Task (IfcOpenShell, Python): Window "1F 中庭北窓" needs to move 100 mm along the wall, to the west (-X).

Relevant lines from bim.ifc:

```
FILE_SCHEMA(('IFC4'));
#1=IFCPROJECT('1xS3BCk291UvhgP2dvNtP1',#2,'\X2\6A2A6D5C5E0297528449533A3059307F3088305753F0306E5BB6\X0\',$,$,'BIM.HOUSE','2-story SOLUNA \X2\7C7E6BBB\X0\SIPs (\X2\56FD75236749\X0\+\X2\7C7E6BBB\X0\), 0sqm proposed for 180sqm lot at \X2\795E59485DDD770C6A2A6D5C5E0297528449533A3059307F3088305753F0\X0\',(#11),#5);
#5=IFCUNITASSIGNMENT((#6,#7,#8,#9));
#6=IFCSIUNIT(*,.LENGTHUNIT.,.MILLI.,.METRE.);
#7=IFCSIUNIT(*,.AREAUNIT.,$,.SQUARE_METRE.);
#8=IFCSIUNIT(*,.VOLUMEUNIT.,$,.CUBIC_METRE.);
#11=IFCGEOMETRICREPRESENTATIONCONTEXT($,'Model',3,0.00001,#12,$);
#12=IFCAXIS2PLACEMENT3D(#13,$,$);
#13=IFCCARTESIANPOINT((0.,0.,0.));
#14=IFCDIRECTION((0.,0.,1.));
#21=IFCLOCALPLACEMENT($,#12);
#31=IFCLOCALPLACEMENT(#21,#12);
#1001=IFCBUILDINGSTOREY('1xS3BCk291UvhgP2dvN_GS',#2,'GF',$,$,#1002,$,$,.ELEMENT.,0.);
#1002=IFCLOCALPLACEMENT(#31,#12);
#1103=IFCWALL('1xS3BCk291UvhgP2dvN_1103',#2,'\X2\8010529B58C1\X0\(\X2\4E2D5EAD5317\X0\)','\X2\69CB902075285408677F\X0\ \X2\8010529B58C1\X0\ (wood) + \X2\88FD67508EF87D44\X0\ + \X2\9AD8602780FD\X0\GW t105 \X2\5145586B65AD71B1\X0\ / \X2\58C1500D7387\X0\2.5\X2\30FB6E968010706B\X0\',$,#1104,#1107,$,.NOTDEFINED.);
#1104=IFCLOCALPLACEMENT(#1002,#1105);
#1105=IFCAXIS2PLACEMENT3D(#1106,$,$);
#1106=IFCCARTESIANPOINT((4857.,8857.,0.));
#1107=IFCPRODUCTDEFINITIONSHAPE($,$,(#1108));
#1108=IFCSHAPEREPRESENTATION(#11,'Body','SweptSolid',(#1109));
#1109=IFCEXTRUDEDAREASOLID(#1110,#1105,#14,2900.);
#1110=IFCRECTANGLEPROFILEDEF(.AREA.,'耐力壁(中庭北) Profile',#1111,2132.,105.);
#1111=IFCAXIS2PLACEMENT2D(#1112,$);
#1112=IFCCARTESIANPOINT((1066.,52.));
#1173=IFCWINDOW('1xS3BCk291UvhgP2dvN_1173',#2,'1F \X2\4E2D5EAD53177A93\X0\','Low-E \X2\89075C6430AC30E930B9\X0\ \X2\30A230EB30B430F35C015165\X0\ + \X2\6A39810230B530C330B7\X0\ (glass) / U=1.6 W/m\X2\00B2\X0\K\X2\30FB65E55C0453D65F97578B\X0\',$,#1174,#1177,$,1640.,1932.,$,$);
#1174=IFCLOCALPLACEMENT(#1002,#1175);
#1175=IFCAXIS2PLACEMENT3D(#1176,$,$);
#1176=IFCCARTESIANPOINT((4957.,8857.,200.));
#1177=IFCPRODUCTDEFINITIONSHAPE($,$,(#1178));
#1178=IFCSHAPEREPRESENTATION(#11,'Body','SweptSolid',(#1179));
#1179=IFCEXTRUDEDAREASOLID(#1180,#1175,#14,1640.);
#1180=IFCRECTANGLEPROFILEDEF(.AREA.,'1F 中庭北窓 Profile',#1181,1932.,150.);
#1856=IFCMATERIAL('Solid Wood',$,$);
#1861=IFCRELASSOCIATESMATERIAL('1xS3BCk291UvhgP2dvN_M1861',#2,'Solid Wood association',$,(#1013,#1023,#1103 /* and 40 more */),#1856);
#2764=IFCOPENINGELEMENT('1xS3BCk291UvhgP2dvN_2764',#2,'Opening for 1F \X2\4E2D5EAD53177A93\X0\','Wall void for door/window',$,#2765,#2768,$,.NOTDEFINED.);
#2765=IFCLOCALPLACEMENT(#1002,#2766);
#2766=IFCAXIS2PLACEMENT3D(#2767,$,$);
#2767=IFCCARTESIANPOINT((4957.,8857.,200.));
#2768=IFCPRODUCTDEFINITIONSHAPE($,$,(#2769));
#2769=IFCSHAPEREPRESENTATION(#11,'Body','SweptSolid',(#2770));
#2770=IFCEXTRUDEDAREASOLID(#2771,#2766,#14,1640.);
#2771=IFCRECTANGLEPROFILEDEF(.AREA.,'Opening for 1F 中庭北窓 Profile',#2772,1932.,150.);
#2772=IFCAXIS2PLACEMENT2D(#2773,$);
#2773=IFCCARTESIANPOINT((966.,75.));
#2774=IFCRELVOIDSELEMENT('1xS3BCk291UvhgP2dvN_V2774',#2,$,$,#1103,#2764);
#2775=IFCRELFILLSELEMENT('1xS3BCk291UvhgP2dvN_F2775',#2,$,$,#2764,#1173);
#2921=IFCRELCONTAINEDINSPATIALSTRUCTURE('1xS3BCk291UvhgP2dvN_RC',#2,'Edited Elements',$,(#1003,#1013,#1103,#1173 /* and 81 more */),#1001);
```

```python
import ifcopenshell
import ifcopenshell.api.geometry
import ifcopenshell.util.placement

model = ifcopenshell.open("bim.ifc")

window = model.by_guid("1xS3BCk291UvhgP2dvN_1173")
opening = window.FillsVoids[0].RelatingOpeningElement
wall = opening.VoidsElements[0].RelatingBuildingElement

wall_matrix = ifcopenshell.util.placement.get_local_placement(wall.ObjectPlacement)
shift = wall_matrix[:3, 0] * -100.0
before = ifcopenshell.util.placement.get_local_placement(window.ObjectPlacement)[:3, 3].copy()

# The window is not placed relative to its opening, so move both.
for product in (opening, window):
    matrix = ifcopenshell.util.placement.get_local_placement(product.ObjectPlacement)
    matrix[:3, 3] += shift
    ifcopenshell.api.geometry.edit_object_placement(model, product=product, matrix=matrix, is_si=False)

after = ifcopenshell.util.placement.get_local_placement(window.ObjectPlacement)[:3, 3]
print("window moved by", (after - before).round(3) + 0.0)

model.write("bim_updated.ifc")
```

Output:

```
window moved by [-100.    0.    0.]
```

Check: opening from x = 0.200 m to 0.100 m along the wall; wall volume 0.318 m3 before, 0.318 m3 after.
